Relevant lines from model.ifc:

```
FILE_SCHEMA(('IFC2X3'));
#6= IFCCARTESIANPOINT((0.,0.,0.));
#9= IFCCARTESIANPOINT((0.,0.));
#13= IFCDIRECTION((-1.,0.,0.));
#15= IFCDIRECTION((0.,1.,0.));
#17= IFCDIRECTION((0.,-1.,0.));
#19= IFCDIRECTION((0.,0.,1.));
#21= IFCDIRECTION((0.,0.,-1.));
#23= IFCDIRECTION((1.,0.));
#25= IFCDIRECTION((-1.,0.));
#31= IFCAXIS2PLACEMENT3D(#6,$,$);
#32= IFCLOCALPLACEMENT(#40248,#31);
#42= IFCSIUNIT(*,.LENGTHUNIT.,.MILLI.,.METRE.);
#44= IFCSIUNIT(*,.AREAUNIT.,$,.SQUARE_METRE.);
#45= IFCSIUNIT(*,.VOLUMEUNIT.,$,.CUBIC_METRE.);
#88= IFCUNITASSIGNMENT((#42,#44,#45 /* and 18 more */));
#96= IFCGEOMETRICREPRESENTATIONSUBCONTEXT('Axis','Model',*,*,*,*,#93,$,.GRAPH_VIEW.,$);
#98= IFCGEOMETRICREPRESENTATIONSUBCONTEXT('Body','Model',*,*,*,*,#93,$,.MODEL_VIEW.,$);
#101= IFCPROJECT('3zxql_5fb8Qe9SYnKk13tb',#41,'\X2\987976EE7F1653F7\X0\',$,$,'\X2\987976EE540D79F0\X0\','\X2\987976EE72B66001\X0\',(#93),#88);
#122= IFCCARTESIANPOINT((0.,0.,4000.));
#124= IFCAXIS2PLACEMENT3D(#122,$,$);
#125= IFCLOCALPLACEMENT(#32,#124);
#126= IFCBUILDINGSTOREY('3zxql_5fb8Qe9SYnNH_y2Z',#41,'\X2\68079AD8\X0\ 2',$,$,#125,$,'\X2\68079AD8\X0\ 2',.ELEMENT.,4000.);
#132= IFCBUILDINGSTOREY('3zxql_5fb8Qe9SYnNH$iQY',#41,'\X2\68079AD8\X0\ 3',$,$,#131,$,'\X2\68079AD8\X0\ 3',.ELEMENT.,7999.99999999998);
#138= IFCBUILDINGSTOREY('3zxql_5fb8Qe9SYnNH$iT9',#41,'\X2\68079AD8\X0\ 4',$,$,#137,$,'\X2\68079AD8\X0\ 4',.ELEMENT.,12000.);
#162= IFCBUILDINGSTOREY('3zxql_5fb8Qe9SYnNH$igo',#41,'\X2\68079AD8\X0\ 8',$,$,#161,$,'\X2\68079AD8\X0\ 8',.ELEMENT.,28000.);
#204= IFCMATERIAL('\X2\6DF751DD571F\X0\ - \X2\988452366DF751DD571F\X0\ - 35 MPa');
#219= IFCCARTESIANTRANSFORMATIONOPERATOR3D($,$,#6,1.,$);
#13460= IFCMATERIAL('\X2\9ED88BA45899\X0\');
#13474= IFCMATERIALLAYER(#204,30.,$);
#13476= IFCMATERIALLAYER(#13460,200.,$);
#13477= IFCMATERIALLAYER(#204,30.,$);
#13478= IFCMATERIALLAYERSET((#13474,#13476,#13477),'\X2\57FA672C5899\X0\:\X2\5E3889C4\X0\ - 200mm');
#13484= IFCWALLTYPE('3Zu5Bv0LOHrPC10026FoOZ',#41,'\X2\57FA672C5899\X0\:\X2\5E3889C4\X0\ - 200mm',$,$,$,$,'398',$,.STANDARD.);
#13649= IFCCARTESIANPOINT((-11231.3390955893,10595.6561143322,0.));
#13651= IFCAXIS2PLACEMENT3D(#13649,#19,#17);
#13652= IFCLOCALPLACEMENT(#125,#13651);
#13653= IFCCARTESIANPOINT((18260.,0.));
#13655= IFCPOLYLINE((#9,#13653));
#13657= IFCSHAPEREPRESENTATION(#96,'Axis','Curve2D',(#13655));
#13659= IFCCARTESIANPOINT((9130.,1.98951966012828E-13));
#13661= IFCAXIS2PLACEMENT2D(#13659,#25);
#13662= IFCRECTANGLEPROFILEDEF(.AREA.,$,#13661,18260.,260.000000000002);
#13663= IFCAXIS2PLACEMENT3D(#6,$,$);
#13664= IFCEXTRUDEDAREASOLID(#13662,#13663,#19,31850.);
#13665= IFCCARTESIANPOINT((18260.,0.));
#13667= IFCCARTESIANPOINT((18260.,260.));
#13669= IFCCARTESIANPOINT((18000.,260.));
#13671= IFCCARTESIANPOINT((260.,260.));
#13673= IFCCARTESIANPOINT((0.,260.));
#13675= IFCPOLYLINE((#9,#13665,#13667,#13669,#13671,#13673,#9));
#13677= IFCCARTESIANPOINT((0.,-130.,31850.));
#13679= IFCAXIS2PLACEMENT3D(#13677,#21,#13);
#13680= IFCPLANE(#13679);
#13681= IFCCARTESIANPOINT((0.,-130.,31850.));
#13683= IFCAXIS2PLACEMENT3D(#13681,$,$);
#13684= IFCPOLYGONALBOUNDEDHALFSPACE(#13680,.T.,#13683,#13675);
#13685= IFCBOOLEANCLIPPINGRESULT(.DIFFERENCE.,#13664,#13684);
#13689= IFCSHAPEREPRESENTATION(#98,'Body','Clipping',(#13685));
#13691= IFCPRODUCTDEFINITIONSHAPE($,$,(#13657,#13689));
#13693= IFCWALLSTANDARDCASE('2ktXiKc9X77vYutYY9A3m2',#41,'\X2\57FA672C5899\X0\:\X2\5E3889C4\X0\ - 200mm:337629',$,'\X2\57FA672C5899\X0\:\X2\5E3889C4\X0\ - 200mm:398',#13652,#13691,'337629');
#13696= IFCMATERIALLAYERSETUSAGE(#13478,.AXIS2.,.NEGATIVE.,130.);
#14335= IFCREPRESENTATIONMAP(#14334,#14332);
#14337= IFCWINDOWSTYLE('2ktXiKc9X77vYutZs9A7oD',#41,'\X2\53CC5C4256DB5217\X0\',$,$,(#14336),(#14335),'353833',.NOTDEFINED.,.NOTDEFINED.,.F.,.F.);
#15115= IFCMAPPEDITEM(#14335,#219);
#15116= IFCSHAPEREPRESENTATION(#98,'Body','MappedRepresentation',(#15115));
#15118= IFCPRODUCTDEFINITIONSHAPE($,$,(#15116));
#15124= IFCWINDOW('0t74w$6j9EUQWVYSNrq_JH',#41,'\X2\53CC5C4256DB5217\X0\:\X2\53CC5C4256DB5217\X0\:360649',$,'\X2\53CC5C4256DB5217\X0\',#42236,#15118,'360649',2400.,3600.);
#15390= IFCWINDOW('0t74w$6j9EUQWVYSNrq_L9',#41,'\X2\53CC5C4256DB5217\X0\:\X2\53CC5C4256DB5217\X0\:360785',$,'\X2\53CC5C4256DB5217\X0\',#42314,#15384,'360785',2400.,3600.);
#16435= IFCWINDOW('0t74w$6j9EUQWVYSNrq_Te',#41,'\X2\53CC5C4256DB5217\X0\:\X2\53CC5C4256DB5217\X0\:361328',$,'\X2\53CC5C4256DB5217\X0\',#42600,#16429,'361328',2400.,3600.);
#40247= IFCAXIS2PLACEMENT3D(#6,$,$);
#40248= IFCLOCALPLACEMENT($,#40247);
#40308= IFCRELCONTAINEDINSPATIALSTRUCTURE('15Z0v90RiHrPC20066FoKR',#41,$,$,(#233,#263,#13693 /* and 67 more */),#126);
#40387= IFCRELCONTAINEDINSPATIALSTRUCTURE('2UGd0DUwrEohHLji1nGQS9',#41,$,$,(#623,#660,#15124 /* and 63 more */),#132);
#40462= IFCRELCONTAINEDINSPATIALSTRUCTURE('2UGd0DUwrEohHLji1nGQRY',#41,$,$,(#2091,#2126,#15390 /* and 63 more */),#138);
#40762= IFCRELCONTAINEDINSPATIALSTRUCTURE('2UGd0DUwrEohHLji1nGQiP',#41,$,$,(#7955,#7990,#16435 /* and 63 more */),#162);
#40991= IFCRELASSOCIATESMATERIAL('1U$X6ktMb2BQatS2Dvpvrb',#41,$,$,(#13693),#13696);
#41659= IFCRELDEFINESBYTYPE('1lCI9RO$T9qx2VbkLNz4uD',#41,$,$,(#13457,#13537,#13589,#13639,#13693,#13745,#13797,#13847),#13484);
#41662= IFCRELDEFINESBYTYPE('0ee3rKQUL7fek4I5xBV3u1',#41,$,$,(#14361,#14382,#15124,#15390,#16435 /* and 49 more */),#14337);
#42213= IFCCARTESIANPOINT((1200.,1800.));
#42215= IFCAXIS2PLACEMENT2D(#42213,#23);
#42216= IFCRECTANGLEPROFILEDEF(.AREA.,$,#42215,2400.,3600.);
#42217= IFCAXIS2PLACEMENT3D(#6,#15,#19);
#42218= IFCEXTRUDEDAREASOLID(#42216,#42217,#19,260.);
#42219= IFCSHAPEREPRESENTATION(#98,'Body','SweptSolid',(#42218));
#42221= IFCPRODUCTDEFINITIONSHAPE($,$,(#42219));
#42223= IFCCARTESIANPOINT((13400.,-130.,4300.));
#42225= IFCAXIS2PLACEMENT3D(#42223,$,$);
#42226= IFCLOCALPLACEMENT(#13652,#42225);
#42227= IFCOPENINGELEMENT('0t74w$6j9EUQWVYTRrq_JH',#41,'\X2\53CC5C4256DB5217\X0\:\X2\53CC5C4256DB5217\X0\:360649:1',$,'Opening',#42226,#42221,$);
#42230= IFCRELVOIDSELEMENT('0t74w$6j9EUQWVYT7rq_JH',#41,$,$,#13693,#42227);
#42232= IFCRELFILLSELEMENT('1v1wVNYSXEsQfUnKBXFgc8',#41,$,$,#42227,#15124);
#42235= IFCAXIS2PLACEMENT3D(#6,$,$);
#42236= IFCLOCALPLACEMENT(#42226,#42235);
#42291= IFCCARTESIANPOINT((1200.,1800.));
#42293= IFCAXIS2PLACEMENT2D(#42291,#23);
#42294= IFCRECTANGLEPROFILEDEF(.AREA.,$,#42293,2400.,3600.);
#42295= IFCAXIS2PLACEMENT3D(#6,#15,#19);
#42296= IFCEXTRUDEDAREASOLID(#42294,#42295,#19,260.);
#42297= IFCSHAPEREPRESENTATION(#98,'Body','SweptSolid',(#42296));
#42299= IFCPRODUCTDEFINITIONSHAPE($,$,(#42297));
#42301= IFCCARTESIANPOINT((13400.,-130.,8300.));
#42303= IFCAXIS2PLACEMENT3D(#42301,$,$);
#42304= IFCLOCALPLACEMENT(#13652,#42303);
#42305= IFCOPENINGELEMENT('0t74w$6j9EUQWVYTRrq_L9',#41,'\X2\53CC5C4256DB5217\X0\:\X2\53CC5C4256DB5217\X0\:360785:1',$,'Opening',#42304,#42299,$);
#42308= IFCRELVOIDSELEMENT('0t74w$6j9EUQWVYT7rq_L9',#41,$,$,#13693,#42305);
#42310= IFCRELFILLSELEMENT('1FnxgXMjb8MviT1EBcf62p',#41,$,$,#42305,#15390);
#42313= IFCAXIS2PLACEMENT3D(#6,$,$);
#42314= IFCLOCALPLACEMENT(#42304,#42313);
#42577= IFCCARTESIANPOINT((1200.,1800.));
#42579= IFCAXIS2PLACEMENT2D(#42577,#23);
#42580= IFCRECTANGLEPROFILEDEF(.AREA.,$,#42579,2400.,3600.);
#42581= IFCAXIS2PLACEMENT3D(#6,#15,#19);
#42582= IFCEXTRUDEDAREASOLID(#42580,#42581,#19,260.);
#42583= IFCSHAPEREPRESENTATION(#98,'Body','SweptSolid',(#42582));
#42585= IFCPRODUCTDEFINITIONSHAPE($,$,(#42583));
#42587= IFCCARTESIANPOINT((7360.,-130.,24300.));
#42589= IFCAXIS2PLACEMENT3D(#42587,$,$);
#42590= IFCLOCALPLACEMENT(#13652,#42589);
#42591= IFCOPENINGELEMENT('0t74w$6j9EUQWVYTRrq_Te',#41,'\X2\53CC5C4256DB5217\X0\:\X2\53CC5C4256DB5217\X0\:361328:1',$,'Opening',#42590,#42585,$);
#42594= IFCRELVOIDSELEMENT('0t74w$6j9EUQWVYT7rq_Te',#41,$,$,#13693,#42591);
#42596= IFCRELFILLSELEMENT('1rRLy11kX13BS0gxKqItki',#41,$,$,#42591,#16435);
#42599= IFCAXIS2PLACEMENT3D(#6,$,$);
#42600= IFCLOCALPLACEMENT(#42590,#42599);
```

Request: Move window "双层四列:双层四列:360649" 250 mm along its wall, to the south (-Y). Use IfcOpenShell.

```python
import ifcopenshell
import ifcopenshell.api.geometry
import ifcopenshell.util.placement
import ifcopenshell.util.unit

model = ifcopenshell.open("model.ifc")
unit_scale = ifcopenshell.util.unit.calculate_unit_scale(model)

window = model.by_id(15124)
opening = window.FillsVoids[0].RelatingOpeningElement
wall = opening.VoidsElements[0].RelatingBuildingElement

wall_matrix = ifcopenshell.util.placement.get_local_placement(wall.ObjectPlacement)
shift = wall_matrix[:3, 0] * 0.25 / unit_scale
before = ifcopenshell.util.placement.get_local_placement(window.ObjectPlacement)[:3, 3].copy()

# The window is placed relative to its opening, so it follows when the opening moves.
matrix = ifcopenshell.util.placement.get_local_placement(opening.ObjectPlacement)
matrix[:3, 3] += shift
ifcopenshell.api.geometry.edit_object_placement(
    model, product=opening, matrix=matrix, is_si=False, should_transform_children=True
)

after = ifcopenshell.util.placement.get_local_placement(window.ObjectPlacement)[:3, 3]
print("window moved by", (after - before).round(3) + 0.0)

model.write("model_rev.ifc")
```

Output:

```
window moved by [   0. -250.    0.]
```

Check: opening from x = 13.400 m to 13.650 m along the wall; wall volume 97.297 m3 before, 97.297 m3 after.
